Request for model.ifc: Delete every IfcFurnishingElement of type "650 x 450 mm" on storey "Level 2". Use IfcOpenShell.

First a look at what the model holds.

```python
import ifcopenshell
import ifcopenshell.util.element

model = ifcopenshell.open("model.ifc")
print(model.schema)
storey = next(s for s in model.by_type("IfcBuildingStorey") if s.Name == "Level 2")
furniture = [e for e in ifcopenshell.util.element.get_decomposition(storey) if e.is_a("IfcFurnishingElement")]
seen = {}
for e in furniture:
    element_type = ifcopenshell.util.element.get_type(e)
    name = element_type.Name if element_type not in (None, e) else None
    seen[name] = seen.get(name, 0) + 1
for name, count in sorted(seen.items(), key=str):
    print(count, "x", name)
```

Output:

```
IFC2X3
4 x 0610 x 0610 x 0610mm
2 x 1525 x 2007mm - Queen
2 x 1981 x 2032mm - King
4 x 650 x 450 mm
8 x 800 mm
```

```python
import ifcopenshell
import ifcopenshell.api.root
import ifcopenshell.util.element

model = ifcopenshell.open("model.ifc")

storey = next(s for s in model.by_type("IfcBuildingStorey") if s.Name == "Level 2")
furniture = [e for e in ifcopenshell.util.element.get_decomposition(storey) if e.is_a("IfcFurnishingElement")]
targets = [e for e in furniture if (t := ifcopenshell.util.element.get_type(e)) not in (None, e) and t.Name == "650 x 450 mm"]

for e in targets:
    ifcopenshell.api.root.remove_product(model, product=e)
print(len(targets), "removed")

model.write("model-out.ifc")
```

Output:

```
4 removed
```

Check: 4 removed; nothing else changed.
